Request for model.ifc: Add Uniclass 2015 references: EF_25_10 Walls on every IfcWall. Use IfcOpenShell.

First a look at what the model holds.

```python
import ifcopenshell

model = ifcopenshell.open("model.ifc")
print(model.schema)
print("classifications:", [c.Name for c in model.by_type("IfcClassification")])
for ifc_class in ("IfcDoor", "IfcRoof", "IfcStair", "IfcWall", "IfcWindow"):
    print(ifc_class, len(model.by_type(ifc_class)))
```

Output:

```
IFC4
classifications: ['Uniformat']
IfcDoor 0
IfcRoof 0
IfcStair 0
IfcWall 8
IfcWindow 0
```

```python
import ifcopenshell
import ifcopenshell.api.classification

model = ifcopenshell.open("model.ifc")

system = ifcopenshell.api.classification.add_classification(model, classification="Uniclass 2015")

codes = {
    "IfcWall": ("EF_25_10", "Walls"),
}
for ifc_class, (code, name) in codes.items():
    products = model.by_type(ifc_class)
    ifcopenshell.api.classification.add_reference(
        model, products=products, classification=system, identification=code, name=name
    )
    print(code, len(products))

model.write("model_edited.ifc")
```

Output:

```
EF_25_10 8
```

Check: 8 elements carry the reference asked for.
